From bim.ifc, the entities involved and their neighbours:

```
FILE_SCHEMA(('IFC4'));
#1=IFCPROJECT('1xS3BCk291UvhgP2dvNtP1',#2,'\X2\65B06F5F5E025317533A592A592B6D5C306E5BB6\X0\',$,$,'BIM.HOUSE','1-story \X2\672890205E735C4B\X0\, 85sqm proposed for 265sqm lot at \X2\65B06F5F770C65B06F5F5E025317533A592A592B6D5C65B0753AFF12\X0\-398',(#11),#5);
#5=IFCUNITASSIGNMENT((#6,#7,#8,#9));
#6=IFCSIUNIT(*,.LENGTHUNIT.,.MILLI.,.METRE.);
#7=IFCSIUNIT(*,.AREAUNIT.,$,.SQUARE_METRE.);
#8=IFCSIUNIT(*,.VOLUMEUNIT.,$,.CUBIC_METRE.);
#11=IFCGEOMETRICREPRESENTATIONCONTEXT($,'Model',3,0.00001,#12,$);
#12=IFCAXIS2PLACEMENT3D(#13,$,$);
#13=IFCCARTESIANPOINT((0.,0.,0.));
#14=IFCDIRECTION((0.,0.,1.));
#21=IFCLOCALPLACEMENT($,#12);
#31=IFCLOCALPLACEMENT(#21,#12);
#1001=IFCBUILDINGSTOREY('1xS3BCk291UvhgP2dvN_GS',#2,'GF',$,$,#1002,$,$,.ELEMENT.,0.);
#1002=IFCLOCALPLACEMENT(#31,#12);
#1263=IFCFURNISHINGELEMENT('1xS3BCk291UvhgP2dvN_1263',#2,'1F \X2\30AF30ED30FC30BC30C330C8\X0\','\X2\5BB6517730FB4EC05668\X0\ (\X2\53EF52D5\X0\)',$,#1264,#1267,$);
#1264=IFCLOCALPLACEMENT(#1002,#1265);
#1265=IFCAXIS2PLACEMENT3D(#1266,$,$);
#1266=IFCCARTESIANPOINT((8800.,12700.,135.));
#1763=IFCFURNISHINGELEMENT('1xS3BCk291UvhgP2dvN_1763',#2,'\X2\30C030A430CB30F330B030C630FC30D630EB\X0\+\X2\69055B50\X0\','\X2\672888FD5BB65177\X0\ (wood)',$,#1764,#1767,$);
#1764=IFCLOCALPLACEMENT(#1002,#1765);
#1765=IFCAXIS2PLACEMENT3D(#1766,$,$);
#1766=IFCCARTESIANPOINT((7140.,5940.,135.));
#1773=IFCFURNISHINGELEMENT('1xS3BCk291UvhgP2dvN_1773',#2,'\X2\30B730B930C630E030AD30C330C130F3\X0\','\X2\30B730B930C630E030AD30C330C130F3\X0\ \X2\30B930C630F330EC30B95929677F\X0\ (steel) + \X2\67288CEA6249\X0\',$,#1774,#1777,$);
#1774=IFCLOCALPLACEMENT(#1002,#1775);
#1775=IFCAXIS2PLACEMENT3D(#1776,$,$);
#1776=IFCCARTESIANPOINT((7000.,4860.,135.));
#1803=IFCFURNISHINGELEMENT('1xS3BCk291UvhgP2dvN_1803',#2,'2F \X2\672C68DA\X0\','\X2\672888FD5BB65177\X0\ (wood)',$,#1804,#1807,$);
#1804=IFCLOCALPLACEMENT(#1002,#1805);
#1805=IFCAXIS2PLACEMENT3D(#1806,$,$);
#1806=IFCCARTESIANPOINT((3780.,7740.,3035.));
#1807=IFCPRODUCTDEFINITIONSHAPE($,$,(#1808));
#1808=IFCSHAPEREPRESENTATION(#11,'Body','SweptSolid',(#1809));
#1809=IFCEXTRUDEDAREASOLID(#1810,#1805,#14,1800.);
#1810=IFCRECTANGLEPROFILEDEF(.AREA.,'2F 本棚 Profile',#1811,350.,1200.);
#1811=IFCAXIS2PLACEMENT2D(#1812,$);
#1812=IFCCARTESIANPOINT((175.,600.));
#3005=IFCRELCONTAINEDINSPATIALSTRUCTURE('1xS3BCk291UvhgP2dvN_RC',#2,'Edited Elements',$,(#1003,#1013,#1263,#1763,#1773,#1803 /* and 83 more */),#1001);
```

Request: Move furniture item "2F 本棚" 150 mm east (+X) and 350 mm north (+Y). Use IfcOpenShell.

```python
import ifcopenshell
import ifcopenshell.api.geometry
import ifcopenshell.util.placement
import ifcopenshell.util.unit

model = ifcopenshell.open("bim.ifc")
unit_scale = ifcopenshell.util.unit.calculate_unit_scale(model)

item = model.by_guid("1xS3BCk291UvhgP2dvN_1803")
matrix = ifcopenshell.util.placement.get_local_placement(item.ObjectPlacement)
matrix[0, 3] += 0.15 / unit_scale
matrix[1, 3] += 0.35 / unit_scale
ifcopenshell.api.geometry.edit_object_placement(model, product=item, matrix=matrix, is_si=False)

print(ifcopenshell.util.placement.get_local_placement(item.ObjectPlacement).round(3) + 0.0)

model.write("bim_edited.ifc")
```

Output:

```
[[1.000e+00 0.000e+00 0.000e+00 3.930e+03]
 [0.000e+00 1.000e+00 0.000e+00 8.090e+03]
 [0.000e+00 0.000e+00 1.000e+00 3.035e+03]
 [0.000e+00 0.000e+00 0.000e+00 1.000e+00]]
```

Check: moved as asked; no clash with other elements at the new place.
